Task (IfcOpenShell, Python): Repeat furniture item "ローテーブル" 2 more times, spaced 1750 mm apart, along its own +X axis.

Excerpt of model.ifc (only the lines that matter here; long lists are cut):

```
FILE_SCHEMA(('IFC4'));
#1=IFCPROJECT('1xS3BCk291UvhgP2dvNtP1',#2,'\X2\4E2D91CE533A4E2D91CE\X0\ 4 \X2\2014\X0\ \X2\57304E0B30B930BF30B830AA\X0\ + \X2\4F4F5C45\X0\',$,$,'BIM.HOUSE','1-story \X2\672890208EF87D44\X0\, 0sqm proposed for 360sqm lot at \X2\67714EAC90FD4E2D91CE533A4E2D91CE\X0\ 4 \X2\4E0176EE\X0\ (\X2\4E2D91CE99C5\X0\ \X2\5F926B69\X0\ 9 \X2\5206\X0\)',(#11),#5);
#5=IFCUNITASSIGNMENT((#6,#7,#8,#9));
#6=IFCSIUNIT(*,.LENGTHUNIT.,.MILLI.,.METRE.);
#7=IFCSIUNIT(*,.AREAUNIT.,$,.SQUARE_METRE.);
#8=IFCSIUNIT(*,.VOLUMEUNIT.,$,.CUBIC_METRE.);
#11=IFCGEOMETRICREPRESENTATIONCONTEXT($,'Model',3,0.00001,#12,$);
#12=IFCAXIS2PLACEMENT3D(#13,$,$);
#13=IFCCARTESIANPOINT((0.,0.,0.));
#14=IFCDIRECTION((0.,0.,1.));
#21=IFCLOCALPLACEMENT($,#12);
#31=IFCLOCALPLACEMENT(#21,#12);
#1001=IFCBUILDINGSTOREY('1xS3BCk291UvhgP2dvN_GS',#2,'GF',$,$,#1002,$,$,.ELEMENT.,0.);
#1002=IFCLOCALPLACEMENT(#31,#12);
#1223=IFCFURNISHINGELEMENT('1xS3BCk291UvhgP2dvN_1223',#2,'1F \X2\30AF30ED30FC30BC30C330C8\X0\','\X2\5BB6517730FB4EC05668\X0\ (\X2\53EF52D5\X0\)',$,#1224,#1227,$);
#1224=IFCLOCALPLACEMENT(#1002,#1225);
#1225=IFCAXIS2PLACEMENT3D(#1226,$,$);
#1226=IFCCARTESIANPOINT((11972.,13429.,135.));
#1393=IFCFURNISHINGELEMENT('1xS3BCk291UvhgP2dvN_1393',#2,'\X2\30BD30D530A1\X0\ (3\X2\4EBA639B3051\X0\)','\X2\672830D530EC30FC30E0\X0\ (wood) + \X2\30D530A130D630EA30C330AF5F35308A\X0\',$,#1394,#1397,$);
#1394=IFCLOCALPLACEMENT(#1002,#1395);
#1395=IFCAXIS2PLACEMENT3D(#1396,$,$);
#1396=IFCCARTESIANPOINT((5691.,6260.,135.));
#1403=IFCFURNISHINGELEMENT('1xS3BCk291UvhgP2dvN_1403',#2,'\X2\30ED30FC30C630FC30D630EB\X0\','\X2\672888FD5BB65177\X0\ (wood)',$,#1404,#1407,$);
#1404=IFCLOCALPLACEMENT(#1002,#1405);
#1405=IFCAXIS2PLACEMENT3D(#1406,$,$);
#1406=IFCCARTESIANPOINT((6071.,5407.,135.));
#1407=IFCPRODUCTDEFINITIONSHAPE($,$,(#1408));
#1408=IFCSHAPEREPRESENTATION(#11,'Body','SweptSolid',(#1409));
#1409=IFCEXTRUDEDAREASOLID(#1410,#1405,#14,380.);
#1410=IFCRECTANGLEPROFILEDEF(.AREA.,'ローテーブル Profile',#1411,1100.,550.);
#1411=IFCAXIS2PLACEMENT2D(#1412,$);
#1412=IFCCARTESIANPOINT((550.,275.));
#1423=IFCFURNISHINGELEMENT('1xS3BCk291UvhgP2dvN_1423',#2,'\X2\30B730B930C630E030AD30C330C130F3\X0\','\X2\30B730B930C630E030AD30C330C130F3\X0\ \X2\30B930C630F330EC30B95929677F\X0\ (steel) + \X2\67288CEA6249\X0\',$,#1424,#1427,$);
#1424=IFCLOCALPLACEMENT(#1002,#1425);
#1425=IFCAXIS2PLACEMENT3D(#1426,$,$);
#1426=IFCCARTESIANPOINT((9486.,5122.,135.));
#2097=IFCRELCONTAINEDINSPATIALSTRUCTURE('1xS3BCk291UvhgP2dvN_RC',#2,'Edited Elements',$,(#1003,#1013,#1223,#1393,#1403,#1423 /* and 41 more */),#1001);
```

```python
import ifcopenshell
import ifcopenshell.api.geometry
import ifcopenshell.api.root
import ifcopenshell.util.element
import ifcopenshell.util.placement

model = ifcopenshell.open("model.ifc")


def reuse_history(source, copy):
    """copy_class also copies each property set's owner history, people and application; keep the originals."""
    for rel in copy.IsDefinedBy:
        if rel.is_a("IfcRelDefinesByProperties") and (history := rel.RelatingPropertyDefinition.OwnerHistory):
            rel.RelatingPropertyDefinition.OwnerHistory = source.OwnerHistory
            ifcopenshell.util.element.remove_deep2(model, history)


source = model.by_guid("1xS3BCk291UvhgP2dvN_1403")
base = ifcopenshell.util.placement.get_local_placement(source.ObjectPlacement)
step = base[:3, 0] * 1750.0

for i in range(1, 3):
    copy = ifcopenshell.api.root.copy_class(model, product=source)
    copy.Representation = ifcopenshell.util.element.copy_deep(
        model, source.Representation, exclude=["IfcGeometricRepresentationContext", "IfcRepresentationMap"]
    )
    reuse_history(source, copy)
    matrix = base.copy()
    matrix[:3, 3] += i * step
    print("added at", matrix[:3, 3].round(3) + 0.0)
    ifcopenshell.api.geometry.edit_object_placement(model, product=copy, matrix=matrix, is_si=False)

model.write("model_rev.ifc")
```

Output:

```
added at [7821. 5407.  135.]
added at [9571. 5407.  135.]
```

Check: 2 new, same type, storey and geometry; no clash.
